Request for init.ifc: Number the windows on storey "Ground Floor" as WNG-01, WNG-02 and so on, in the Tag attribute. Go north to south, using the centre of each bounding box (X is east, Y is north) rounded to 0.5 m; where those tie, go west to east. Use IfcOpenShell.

First a look at what the model holds.

```python
import ifcopenshell
import ifcopenshell.util.element
import ifcopenshell.util.placement

model = ifcopenshell.open("init.ifc")
print(model.schema)
storey = next(s for s in model.by_type("IfcBuildingStorey") if s.Name == "Ground Floor")
windows = [e for e in ifcopenshell.util.element.get_decomposition(storey) if e.is_a("IfcWindow")]
for e in sorted(windows, key=lambda e: e.id()):
    origin = ifcopenshell.util.placement.get_local_placement(e.ObjectPlacement)[:3, 3]
    print(e.id(), e.Tag, e.Name, origin.round(2) + 0.0, sep=" | ")
```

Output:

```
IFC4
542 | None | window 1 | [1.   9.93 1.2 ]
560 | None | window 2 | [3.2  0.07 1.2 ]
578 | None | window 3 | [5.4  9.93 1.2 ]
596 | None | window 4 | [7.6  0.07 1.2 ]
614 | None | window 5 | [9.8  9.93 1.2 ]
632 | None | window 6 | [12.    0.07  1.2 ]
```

```python
import ifcopenshell
import ifcopenshell.geom
import ifcopenshell.util.element
import ifcopenshell.util.shape

model = ifcopenshell.open("init.ifc")
settings = ifcopenshell.geom.settings()
settings.set("use-world-coords", True)


def centre(element):
    shape = ifcopenshell.geom.create_shape(settings, element)
    return ifcopenshell.util.shape.get_bbox_centroid(shape.geometry)


storey = next(s for s in model.by_type("IfcBuildingStorey") if s.Name == "Ground Floor")
windows = [e for e in ifcopenshell.util.element.get_decomposition(storey) if e.is_a("IfcWindow")]

# Insertion points can sit at a corner or the storey origin, so sort by the geometry (in metres).
centres = {e: centre(e) for e in windows}
windows.sort(key=lambda e: (-round(centres[e][1] / 0.5), centres[e][0]))

for i, e in enumerate(windows, start=1):
    number = f"WNG-{i:02d}"
    e.Tag = number
    print(e.id(), number)

model.write("init_edited.ifc")
```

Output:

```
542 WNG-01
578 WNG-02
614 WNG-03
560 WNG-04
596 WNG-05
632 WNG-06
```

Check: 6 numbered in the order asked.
